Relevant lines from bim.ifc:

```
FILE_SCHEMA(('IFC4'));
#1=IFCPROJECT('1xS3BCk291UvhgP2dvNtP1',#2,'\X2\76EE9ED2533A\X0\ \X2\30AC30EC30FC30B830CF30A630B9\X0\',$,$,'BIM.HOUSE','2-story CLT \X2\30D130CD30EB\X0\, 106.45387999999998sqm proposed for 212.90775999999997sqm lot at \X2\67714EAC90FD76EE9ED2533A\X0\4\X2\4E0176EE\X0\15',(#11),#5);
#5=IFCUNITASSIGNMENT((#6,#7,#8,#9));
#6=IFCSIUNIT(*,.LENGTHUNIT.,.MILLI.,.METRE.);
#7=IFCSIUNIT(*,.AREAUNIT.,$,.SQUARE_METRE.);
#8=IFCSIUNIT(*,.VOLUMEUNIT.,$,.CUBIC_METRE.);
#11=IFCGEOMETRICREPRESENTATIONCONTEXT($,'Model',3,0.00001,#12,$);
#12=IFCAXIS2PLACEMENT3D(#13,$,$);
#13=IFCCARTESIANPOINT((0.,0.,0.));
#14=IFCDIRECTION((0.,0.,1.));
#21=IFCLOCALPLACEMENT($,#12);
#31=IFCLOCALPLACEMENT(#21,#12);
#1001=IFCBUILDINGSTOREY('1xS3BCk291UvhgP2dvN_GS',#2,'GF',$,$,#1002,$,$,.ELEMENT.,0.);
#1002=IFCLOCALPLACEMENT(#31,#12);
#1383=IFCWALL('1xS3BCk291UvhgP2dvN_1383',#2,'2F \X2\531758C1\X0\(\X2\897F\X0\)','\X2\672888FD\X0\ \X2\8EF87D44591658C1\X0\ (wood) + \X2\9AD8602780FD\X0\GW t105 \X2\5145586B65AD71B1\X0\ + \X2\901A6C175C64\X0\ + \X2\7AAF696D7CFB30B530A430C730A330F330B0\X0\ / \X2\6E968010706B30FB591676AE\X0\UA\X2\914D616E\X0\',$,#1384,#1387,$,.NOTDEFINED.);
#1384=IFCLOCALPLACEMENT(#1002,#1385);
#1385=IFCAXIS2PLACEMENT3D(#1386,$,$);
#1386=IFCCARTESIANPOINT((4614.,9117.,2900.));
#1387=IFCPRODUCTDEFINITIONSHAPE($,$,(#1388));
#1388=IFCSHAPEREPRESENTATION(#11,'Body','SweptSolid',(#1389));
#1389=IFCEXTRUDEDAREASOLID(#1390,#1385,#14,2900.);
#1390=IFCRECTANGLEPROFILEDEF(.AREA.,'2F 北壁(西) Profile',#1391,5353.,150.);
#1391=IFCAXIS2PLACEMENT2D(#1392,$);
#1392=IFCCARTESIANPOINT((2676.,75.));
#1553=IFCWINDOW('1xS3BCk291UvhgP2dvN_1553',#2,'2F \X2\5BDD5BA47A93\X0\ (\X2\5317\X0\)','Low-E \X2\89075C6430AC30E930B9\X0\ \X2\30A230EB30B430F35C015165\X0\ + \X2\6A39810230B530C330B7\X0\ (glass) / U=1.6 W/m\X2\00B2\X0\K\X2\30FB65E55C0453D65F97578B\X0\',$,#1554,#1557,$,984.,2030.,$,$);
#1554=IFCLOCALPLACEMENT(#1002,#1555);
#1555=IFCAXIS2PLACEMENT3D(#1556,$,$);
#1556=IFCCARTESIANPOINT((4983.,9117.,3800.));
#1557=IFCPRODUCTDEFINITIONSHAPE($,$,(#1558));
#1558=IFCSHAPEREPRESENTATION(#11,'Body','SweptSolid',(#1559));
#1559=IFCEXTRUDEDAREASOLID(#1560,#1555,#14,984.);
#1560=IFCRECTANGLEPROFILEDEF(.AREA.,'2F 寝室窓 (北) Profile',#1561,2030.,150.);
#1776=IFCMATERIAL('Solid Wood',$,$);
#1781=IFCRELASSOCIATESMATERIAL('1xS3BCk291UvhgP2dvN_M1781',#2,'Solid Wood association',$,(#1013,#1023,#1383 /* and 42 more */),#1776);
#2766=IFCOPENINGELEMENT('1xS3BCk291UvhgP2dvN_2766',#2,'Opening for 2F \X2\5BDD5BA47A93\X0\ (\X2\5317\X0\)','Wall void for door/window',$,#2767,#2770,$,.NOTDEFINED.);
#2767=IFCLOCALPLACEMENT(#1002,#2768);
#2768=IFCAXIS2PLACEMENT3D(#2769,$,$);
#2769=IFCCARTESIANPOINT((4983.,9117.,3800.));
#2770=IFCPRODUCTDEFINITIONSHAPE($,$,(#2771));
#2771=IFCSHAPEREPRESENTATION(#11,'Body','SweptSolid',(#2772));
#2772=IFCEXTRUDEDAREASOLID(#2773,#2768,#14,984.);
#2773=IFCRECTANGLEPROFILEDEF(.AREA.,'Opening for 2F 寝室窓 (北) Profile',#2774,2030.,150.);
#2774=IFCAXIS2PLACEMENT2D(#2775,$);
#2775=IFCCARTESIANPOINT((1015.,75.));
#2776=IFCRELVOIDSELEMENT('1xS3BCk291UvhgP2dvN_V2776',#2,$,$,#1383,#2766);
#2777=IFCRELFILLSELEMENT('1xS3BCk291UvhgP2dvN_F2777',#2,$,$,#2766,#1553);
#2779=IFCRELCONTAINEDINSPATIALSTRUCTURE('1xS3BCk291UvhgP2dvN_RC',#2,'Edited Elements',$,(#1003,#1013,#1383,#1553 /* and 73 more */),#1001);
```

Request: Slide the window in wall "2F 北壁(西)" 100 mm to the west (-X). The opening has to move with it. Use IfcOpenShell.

```python
import ifcopenshell
import ifcopenshell.api.geometry
import ifcopenshell.util.placement

model = ifcopenshell.open("bim.ifc")

window = model.by_id(1553)
opening = window.FillsVoids[0].RelatingOpeningElement
wall = opening.VoidsElements[0].RelatingBuildingElement

wall_matrix = ifcopenshell.util.placement.get_local_placement(wall.ObjectPlacement)
shift = wall_matrix[:3, 0] * -100.0
before = ifcopenshell.util.placement.get_local_placement(window.ObjectPlacement)[:3, 3].copy()

# The window is not placed relative to its opening, so move both.
for product in (opening, window):
    matrix = ifcopenshell.util.placement.get_local_placement(product.ObjectPlacement)
    matrix[:3, 3] += shift
    ifcopenshell.api.geometry.edit_object_placement(model, product=product, matrix=matrix, is_si=False)

after = ifcopenshell.util.placement.get_local_placement(window.ObjectPlacement)[:3, 3]
print("window moved by", (after - before).round(3) + 0.0)

model.write("bim_updated.ifc")
```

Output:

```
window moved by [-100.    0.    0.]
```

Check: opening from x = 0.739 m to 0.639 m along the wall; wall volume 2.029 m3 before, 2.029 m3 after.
